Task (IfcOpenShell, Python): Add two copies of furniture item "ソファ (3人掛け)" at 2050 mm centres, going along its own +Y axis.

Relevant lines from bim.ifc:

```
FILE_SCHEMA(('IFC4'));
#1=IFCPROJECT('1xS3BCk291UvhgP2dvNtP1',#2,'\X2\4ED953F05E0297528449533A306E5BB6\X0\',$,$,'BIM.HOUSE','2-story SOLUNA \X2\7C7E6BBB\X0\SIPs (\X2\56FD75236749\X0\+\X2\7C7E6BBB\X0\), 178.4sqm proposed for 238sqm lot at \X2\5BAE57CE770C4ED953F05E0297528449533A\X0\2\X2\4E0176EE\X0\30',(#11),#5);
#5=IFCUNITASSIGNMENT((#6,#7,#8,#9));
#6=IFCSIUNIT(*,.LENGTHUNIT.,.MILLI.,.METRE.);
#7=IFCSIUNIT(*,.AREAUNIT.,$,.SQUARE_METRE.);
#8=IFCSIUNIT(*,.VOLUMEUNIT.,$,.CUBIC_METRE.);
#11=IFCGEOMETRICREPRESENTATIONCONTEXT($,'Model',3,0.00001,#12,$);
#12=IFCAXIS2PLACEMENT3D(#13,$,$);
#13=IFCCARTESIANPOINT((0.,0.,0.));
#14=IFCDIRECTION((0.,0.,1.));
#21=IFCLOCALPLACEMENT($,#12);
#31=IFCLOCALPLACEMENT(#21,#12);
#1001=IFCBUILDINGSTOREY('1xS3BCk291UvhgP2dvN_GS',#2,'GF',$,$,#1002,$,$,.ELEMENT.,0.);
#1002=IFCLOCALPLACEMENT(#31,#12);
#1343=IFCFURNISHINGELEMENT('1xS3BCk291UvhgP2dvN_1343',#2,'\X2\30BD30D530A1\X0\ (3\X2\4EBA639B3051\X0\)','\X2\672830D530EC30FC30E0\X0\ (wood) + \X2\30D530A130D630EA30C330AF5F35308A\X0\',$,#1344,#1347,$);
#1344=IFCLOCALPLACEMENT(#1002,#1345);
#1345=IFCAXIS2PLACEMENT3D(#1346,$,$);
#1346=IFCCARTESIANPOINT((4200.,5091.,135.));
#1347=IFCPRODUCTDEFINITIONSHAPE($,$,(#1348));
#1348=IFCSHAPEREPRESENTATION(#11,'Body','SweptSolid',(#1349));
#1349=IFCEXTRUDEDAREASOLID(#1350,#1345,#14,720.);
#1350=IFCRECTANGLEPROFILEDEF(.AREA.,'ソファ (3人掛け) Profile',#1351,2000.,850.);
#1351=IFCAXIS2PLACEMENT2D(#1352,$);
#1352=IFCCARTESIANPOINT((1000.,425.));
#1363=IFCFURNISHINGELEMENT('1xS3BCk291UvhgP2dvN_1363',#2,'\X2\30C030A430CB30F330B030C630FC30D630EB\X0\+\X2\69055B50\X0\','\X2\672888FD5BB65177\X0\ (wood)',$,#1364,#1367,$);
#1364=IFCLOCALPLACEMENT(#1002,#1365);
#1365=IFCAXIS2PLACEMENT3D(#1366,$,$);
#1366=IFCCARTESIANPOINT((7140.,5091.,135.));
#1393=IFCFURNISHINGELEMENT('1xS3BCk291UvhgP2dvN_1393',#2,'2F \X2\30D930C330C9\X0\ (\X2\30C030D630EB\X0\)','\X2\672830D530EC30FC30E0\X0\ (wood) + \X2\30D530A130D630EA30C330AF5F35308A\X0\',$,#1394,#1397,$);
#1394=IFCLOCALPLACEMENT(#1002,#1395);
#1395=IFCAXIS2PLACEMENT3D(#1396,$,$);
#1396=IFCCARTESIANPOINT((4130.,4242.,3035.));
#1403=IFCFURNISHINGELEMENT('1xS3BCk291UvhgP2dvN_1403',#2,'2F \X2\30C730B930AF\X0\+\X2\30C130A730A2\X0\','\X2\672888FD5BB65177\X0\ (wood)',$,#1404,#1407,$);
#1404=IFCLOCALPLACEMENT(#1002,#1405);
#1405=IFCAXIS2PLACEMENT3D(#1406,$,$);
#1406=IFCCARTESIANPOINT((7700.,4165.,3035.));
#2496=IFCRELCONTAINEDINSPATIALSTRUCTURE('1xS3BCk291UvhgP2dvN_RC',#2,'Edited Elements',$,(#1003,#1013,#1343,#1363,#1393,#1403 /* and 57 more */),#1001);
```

```python
import ifcopenshell
import ifcopenshell.api.geometry
import ifcopenshell.api.root
import ifcopenshell.util.element
import ifcopenshell.util.placement

model = ifcopenshell.open("bim.ifc")


def reuse_history(source, copy):
    """copy_class also copies each property set's owner history, people and application; keep the originals."""
    for rel in copy.IsDefinedBy:
        if rel.is_a("IfcRelDefinesByProperties") and (history := rel.RelatingPropertyDefinition.OwnerHistory):
            rel.RelatingPropertyDefinition.OwnerHistory = source.OwnerHistory
            ifcopenshell.util.element.remove_deep2(model, history)


source = model.by_id(1343)
base = ifcopenshell.util.placement.get_local_placement(source.ObjectPlacement)
step = base[:3, 1] * 2050.0

for i in range(1, 3):
    copy = ifcopenshell.api.root.copy_class(model, product=source)
    copy.Representation = ifcopenshell.util.element.copy_deep(
        model, source.Representation, exclude=["IfcGeometricRepresentationContext", "IfcRepresentationMap"]
    )
    reuse_history(source, copy)
    matrix = base.copy()
    matrix[:3, 3] += i * step
    print("added at", matrix[:3, 3].round(3) + 0.0)
    ifcopenshell.api.geometry.edit_object_placement(model, product=copy, matrix=matrix, is_si=False)

model.write("bim_updated.ifc")
```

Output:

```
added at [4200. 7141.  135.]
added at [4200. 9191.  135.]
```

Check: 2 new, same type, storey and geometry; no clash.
